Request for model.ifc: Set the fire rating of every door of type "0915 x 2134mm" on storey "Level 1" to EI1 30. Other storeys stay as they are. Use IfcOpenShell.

First a look at what the model holds.

```python
import ifcopenshell
import ifcopenshell.util.element

model = ifcopenshell.open("model.ifc")
print(model.schema)
storey = next(s for s in model.by_type("IfcBuildingStorey") if s.Name == "Level 1")
doors = [e for e in ifcopenshell.util.element.get_decomposition(storey) if e.is_a("IfcDoor")]
seen = {}
for e in doors:
    element_type = ifcopenshell.util.element.get_type(e)
    key = (element_type.Name if element_type != e and element_type else None, ifcopenshell.util.element.get_pset(e, "Pset_DoorCommon", "FireRating"))
    seen[key] = seen.get(key, 0) + 1
for (name, value), count in sorted(seen.items(), key=str):
    print(count, "x", name, "|", value)
```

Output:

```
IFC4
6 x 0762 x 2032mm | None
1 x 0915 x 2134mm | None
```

```python
import ifcopenshell
import ifcopenshell.api.pset
import ifcopenshell.util.element

model = ifcopenshell.open("model.ifc")

storey = next(s for s in model.by_type("IfcBuildingStorey") if s.Name == "Level 1")
doors = [e for e in ifcopenshell.util.element.get_decomposition(storey) if e.is_a("IfcDoor")]

count = 0
for e in doors:
    element_type = ifcopenshell.util.element.get_type(e)
    if element_type in (None, e) or element_type.Name != "0915 x 2134mm":
        continue
    # add_pset returns the element's existing set when there is one.
    pset = ifcopenshell.api.pset.add_pset(model, product=e, name="Pset_DoorCommon")
    ifcopenshell.api.pset.edit_pset(model, pset=pset, properties={"FireRating": "EI1 30"})
    count += 1

print(count, "doors updated")

model.write("model_edited.ifc")
```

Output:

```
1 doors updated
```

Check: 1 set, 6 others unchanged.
